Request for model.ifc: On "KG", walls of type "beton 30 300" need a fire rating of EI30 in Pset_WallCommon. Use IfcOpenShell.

First a look at what the model holds.

```python
import ifcopenshell
import ifcopenshell.util.element

model = ifcopenshell.open("model.ifc")
print(model.schema)
storey = next(s for s in model.by_type("IfcBuildingStorey") if s.Name == "KG")
walls = [e for e in ifcopenshell.util.element.get_decomposition(storey) if e.is_a("IfcWall")]
seen = {}
for e in walls:
    element_type = ifcopenshell.util.element.get_type(e)
    key = (element_type.Name if element_type != e and element_type else None, ifcopenshell.util.element.get_pset(e, "Pset_WallCommon", "FireRating"))
    seen[key] = seen.get(key, 0) + 1
for (name, value), count in sorted(seen.items(), key=str):
    print(count, "x", name, "|", value)
```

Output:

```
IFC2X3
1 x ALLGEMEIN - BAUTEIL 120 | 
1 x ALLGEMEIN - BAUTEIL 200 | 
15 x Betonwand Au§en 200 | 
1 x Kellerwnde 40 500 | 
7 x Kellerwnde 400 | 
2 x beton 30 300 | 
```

```python
import ifcopenshell
import ifcopenshell.api.pset
import ifcopenshell.util.element

model = ifcopenshell.open("model.ifc")

storey = next(s for s in model.by_type("IfcBuildingStorey") if s.Name == "KG")
walls = [e for e in ifcopenshell.util.element.get_decomposition(storey) if e.is_a("IfcWall")]

count = 0
for e in walls:
    element_type = ifcopenshell.util.element.get_type(e)
    if element_type in (None, e) or element_type.Name != "beton 30 300":
        continue
    # add_pset returns the element's existing set when there is one.
    pset = ifcopenshell.api.pset.add_pset(model, product=e, name="Pset_WallCommon")
    ifcopenshell.api.pset.edit_pset(model, pset=pset, properties={"FireRating": "EI30"})
    count += 1

print(count, "walls updated")

model.write("model_rev.ifc")
```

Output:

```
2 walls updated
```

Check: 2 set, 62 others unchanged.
